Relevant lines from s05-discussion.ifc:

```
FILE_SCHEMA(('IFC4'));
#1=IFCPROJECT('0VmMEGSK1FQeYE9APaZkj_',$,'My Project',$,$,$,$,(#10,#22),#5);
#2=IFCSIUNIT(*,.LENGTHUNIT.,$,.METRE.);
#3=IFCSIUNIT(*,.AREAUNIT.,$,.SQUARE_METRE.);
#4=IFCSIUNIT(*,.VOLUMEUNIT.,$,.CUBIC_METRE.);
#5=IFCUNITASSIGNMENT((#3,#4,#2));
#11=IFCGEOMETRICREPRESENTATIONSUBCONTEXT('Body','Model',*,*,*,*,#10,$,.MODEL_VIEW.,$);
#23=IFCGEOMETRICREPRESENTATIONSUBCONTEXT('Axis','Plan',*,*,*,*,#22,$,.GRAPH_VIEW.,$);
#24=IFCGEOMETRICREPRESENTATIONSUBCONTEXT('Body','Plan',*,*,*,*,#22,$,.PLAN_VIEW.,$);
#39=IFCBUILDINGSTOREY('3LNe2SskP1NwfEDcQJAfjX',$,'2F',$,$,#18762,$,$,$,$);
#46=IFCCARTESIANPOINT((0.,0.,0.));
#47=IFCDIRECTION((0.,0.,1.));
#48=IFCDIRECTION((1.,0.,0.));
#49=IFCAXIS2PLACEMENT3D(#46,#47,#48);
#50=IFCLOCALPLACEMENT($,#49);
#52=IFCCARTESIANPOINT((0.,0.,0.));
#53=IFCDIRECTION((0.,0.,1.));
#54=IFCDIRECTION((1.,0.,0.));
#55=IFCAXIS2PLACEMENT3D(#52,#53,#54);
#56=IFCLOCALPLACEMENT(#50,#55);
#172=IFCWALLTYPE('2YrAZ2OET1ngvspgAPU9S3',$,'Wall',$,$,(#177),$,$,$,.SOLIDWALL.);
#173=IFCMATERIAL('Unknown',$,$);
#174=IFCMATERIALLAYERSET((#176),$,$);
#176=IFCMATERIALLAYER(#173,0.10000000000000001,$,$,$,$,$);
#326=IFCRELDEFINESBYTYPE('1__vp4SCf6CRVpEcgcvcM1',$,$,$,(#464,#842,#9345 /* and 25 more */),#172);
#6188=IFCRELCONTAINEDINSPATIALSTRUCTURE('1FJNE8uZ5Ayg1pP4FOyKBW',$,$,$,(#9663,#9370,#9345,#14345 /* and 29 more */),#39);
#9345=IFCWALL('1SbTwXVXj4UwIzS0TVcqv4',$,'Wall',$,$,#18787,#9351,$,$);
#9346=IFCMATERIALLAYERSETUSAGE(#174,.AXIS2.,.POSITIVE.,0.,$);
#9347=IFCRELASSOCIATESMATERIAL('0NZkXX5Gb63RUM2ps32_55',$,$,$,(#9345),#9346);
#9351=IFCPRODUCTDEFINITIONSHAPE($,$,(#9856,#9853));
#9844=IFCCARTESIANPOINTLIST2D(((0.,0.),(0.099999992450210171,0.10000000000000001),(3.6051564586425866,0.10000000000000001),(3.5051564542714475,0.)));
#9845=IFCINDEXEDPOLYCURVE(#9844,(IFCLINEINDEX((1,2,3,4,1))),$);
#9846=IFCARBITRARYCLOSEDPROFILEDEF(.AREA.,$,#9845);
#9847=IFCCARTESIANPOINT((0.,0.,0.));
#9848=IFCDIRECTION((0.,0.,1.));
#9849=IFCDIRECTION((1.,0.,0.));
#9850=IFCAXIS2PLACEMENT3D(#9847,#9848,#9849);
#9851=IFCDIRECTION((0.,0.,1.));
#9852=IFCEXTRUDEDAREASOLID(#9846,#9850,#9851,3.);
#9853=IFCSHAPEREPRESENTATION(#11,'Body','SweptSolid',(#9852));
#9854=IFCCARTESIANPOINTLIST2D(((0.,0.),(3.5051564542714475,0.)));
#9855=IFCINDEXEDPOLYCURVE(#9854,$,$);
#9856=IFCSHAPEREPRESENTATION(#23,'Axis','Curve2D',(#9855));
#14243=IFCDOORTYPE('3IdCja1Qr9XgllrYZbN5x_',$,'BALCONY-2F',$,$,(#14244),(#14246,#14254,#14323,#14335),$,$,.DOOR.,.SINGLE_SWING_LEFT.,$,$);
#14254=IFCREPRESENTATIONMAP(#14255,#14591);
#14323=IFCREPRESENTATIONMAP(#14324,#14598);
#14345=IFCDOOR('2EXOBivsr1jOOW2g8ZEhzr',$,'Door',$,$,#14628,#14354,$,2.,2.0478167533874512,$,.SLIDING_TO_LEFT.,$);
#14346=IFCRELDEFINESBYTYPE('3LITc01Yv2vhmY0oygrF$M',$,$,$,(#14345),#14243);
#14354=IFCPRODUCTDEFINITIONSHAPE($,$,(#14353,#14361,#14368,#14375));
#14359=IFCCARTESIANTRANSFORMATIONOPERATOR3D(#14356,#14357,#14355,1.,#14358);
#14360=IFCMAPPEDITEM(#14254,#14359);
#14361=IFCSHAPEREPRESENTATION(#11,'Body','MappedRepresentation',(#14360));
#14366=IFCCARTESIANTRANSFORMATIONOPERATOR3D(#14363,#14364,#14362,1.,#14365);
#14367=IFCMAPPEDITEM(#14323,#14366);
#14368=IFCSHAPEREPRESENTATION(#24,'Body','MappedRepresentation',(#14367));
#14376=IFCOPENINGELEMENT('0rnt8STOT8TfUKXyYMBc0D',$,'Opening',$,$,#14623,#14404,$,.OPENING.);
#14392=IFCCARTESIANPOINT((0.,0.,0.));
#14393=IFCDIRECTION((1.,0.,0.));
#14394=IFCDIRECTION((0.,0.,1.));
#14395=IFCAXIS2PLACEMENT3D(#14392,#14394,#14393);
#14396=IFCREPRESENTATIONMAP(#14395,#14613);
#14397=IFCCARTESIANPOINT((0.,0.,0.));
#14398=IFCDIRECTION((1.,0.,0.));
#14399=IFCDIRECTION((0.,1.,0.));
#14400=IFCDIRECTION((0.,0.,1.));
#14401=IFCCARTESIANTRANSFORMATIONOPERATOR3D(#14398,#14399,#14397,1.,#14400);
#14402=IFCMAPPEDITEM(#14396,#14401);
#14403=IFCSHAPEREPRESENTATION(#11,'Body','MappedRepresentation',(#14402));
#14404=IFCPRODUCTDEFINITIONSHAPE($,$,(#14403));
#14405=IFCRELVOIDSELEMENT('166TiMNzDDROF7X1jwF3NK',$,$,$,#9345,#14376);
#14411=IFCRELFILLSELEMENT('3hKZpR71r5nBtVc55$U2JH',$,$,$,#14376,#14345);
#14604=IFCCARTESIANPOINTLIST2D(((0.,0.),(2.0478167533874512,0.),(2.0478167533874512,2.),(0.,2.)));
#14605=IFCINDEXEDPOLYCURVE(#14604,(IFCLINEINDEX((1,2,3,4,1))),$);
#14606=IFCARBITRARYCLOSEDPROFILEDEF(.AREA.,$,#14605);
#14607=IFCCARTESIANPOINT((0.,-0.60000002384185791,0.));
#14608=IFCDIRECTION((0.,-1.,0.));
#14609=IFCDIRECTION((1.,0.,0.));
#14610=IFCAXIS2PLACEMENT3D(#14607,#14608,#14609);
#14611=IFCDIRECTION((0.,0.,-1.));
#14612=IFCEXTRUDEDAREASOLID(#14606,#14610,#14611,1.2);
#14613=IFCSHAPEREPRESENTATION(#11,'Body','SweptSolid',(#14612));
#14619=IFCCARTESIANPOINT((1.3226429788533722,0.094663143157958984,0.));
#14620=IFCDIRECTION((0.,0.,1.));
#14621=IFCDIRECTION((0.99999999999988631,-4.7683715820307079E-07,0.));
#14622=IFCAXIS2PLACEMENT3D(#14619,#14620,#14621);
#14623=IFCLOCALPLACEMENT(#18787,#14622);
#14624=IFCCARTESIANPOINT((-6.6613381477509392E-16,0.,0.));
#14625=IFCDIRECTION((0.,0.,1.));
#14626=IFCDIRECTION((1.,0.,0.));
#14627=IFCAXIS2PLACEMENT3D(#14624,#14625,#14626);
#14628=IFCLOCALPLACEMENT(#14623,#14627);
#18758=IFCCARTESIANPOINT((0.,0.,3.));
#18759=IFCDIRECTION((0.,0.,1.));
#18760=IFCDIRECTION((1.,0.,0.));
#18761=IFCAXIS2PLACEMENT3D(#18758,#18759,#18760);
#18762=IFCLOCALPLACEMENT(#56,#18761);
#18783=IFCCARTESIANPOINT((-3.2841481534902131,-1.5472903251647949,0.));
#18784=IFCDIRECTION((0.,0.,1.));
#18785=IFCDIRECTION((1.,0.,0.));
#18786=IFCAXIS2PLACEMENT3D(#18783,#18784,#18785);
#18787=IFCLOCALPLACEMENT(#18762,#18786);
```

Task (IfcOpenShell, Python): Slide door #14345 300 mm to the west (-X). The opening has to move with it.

```python
import ifcopenshell
import ifcopenshell.api.geometry
import ifcopenshell.util.placement
import ifcopenshell.util.unit

model = ifcopenshell.open("s05-discussion.ifc")
unit_scale = ifcopenshell.util.unit.calculate_unit_scale(model)

door = model.by_guid("2EXOBivsr1jOOW2g8ZEhzr")
opening = door.FillsVoids[0].RelatingOpeningElement
wall = opening.VoidsElements[0].RelatingBuildingElement

wall_matrix = ifcopenshell.util.placement.get_local_placement(wall.ObjectPlacement)
shift = wall_matrix[:3, 0] * -0.3 / unit_scale
before = ifcopenshell.util.placement.get_local_placement(door.ObjectPlacement)[:3, 3].copy()

# The door is placed relative to its opening, so it follows when the opening moves.
matrix = ifcopenshell.util.placement.get_local_placement(opening.ObjectPlacement)
matrix[:3, 3] += shift
ifcopenshell.api.geometry.edit_object_placement(
    model, product=opening, matrix=matrix, is_si=False, should_transform_children=True
)

after = ifcopenshell.util.placement.get_local_placement(door.ObjectPlacement)[:3, 3]
print("door moved by", (after - before).round(3) + 0.0)

model.write("s05-discussion_updated.ifc")
```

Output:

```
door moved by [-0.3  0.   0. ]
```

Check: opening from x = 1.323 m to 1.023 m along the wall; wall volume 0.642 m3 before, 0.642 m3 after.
